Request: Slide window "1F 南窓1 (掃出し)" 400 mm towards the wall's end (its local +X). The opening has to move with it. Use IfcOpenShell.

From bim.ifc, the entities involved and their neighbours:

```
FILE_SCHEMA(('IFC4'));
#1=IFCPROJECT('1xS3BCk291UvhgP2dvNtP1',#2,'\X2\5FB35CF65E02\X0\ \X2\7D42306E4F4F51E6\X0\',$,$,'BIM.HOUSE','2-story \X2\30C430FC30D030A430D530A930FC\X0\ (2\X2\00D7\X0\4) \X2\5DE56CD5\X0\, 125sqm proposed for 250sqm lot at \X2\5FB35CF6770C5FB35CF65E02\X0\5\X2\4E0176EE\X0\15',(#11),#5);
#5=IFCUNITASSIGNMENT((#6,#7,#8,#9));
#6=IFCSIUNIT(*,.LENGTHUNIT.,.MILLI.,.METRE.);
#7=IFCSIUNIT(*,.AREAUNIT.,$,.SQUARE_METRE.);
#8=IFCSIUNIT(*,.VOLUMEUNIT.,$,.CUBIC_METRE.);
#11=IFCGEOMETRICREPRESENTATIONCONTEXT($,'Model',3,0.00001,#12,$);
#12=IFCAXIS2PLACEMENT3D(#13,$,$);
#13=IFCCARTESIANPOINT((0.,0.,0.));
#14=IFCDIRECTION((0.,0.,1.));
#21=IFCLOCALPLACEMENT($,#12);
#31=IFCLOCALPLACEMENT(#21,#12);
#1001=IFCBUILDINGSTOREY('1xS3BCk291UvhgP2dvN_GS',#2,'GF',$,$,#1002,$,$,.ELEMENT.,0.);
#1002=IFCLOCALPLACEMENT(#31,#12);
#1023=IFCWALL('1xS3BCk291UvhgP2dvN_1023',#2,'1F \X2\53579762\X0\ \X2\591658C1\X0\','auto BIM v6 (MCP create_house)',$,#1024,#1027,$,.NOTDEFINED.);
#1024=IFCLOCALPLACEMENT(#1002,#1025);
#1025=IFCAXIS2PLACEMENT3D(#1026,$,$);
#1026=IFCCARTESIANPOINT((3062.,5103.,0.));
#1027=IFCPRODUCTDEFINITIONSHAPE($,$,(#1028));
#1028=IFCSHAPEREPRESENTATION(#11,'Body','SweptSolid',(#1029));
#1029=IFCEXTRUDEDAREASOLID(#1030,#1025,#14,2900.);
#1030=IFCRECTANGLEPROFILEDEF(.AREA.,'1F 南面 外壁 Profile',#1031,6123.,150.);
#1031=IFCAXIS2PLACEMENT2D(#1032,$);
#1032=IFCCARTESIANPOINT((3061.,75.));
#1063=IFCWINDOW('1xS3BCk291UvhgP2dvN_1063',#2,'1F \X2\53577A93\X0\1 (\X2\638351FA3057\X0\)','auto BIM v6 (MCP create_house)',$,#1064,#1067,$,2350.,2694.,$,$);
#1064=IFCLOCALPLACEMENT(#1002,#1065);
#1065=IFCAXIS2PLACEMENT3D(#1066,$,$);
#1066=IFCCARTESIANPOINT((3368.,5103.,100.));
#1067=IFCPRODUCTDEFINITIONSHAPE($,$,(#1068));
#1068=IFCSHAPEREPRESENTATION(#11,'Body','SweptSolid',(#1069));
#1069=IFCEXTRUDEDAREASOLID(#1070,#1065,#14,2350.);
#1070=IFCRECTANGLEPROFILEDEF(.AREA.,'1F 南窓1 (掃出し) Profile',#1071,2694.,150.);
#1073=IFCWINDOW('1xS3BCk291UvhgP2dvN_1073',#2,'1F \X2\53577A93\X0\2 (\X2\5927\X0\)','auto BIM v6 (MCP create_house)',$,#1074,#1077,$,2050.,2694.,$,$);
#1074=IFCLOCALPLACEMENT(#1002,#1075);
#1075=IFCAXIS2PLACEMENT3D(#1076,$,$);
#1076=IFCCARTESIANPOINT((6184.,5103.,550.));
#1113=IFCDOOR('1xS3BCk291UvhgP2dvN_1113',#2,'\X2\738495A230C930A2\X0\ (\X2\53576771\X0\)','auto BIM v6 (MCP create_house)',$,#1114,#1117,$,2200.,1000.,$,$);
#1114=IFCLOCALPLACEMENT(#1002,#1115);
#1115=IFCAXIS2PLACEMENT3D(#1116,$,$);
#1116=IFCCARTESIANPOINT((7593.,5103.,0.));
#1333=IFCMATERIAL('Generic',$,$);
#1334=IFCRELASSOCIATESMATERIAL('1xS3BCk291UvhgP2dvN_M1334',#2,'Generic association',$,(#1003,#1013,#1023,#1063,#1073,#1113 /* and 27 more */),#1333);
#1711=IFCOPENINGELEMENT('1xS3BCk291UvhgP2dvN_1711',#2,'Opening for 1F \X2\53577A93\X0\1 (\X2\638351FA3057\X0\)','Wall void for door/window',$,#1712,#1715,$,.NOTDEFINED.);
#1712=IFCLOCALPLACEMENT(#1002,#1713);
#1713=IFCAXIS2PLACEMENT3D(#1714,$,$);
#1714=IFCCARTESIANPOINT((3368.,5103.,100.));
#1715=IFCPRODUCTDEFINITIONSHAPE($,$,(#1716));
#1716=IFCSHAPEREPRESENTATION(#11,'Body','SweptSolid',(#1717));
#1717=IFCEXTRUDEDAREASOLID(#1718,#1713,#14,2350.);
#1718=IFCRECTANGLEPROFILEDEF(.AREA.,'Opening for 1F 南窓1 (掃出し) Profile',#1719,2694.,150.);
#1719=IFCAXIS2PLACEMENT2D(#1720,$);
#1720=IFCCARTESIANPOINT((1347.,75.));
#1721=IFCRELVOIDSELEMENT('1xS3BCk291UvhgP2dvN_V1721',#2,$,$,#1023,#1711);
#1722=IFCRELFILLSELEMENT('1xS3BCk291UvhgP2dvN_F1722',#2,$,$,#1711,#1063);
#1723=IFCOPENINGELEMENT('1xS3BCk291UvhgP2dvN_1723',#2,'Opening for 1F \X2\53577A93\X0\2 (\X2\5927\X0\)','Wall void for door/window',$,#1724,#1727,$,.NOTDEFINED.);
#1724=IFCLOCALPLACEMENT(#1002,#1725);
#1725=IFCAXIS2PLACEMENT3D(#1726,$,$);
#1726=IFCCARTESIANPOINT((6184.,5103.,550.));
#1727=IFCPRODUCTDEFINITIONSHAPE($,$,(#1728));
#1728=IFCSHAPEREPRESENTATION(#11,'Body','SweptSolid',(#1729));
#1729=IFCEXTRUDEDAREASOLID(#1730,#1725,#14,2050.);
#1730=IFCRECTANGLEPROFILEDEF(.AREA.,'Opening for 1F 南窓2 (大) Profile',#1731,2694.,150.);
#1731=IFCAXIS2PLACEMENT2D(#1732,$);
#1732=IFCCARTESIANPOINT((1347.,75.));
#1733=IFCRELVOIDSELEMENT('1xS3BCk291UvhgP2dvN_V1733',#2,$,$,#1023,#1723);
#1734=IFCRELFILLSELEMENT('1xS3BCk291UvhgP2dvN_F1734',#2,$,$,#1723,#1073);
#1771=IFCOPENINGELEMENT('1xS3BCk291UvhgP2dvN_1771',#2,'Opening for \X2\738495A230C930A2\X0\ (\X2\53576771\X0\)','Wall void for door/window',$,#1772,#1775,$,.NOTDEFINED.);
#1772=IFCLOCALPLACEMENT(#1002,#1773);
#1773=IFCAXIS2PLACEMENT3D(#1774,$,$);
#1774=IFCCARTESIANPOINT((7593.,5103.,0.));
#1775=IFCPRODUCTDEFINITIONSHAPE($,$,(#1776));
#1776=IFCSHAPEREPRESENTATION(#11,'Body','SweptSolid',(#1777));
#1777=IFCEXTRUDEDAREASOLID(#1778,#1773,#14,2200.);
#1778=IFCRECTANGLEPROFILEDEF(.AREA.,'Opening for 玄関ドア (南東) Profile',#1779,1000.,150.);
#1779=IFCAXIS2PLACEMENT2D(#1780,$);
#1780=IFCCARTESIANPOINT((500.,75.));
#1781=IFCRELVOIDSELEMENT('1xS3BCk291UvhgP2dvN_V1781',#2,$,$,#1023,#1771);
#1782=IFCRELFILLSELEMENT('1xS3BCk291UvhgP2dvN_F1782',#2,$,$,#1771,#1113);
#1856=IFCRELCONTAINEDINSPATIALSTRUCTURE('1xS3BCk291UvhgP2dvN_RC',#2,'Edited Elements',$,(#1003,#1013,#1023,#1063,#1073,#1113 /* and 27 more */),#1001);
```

```python
import ifcopenshell
import ifcopenshell.api.geometry
import ifcopenshell.util.placement

model = ifcopenshell.open("bim.ifc")

window = model.by_id(1063)
opening = window.FillsVoids[0].RelatingOpeningElement
wall = opening.VoidsElements[0].RelatingBuildingElement

wall_matrix = ifcopenshell.util.placement.get_local_placement(wall.ObjectPlacement)
shift = wall_matrix[:3, 0] * 400.0
before = ifcopenshell.util.placement.get_local_placement(window.ObjectPlacement)[:3, 3].copy()

# The window is not placed relative to its opening, so move both.
for product in (opening, window):
    matrix = ifcopenshell.util.placement.get_local_placement(product.ObjectPlacement)
    matrix[:3, 3] += shift
    ifcopenshell.api.geometry.edit_object_placement(model, product=product, matrix=matrix, is_si=False)

after = ifcopenshell.util.placement.get_local_placement(window.ObjectPlacement)[:3, 3]
print("window moved by", (after - before).round(3) + 0.0)

model.write("bim_rev.ifc")
```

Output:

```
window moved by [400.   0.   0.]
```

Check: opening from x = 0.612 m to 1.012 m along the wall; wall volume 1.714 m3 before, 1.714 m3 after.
